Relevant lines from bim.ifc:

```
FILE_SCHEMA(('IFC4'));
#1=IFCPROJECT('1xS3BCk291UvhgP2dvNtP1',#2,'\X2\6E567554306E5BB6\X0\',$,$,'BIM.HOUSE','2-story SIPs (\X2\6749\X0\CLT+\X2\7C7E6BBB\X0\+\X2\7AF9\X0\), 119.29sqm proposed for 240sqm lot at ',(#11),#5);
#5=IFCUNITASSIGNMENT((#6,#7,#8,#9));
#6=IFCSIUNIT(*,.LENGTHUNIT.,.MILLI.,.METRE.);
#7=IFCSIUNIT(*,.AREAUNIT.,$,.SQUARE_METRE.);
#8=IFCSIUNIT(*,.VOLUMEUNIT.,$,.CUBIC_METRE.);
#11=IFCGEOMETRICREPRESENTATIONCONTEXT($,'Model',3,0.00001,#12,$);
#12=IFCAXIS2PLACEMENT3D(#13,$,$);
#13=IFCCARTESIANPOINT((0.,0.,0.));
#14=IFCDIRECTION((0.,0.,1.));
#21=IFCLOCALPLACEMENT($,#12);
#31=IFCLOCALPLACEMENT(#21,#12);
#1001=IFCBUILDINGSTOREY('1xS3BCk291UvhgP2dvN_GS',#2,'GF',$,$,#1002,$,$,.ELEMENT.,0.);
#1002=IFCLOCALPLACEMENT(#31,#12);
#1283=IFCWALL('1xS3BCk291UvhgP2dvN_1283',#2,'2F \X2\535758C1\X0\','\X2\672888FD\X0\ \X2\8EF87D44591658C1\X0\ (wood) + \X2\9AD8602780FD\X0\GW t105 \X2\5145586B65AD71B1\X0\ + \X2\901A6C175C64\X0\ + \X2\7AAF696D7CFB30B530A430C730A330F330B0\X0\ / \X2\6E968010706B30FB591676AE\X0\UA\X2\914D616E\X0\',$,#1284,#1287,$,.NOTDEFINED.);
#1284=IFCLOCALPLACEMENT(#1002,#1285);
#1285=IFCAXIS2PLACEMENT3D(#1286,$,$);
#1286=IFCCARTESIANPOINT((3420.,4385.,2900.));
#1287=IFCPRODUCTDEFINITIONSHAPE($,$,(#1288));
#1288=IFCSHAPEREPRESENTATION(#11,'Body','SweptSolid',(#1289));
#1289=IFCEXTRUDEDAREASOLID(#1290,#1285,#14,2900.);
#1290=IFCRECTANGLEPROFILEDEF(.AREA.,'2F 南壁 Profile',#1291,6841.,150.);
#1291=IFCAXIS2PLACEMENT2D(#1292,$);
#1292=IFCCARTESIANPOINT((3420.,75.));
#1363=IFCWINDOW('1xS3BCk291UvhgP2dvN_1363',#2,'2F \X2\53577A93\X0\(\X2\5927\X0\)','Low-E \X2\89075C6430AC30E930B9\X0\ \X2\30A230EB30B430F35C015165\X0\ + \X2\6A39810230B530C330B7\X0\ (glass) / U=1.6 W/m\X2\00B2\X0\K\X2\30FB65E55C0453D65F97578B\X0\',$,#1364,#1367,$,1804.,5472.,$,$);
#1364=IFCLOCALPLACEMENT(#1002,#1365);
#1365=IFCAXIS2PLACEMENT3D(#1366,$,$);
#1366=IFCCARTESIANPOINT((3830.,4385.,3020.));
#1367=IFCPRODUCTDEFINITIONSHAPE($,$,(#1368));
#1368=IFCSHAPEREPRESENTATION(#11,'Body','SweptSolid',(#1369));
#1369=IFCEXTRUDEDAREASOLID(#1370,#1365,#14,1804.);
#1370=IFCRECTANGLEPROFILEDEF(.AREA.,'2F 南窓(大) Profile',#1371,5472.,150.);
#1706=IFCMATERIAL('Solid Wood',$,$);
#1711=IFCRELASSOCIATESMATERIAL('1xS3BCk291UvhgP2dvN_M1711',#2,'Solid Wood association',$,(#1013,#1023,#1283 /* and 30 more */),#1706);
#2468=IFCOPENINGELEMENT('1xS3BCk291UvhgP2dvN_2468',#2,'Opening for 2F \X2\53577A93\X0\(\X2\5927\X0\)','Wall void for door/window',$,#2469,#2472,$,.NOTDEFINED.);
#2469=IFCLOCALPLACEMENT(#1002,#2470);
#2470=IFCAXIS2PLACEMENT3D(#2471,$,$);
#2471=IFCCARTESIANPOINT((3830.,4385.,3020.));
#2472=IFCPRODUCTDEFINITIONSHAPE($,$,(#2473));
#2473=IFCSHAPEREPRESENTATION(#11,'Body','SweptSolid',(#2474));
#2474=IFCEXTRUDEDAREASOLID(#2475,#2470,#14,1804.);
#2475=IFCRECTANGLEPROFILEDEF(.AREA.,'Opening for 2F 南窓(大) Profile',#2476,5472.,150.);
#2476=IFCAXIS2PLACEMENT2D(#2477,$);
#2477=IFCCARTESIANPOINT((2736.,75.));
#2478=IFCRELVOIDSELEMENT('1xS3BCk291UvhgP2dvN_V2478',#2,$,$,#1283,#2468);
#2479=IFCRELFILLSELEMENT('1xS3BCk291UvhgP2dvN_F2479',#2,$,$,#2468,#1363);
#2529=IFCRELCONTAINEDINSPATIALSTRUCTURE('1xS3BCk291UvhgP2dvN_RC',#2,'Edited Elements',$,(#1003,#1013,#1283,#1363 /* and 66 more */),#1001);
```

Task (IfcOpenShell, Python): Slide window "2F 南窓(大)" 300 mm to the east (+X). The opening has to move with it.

```python
import ifcopenshell
import ifcopenshell.api.geometry
import ifcopenshell.util.placement
import ifcopenshell.util.unit

model = ifcopenshell.open("bim.ifc")
unit_scale = ifcopenshell.util.unit.calculate_unit_scale(model)

window = model.by_guid("1xS3BCk291UvhgP2dvN_1363")
opening = window.FillsVoids[0].RelatingOpeningElement
wall = opening.VoidsElements[0].RelatingBuildingElement

wall_matrix = ifcopenshell.util.placement.get_local_placement(wall.ObjectPlacement)
shift = wall_matrix[:3, 0] * 0.3 / unit_scale
before = ifcopenshell.util.placement.get_local_placement(window.ObjectPlacement)[:3, 3].copy()

# The window is not placed relative to its opening, so move both.
for product in (opening, window):
    matrix = ifcopenshell.util.placement.get_local_placement(product.ObjectPlacement)
    matrix[:3, 3] += shift
    ifcopenshell.api.geometry.edit_object_placement(model, product=product, matrix=matrix, is_si=False)

after = ifcopenshell.util.placement.get_local_placement(window.ObjectPlacement)[:3, 3]
print("window moved by", (after - before).round(3) + 0.0)

model.write("bim_edited.ifc")
```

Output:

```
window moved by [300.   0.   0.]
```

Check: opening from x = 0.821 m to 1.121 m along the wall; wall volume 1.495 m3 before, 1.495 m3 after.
